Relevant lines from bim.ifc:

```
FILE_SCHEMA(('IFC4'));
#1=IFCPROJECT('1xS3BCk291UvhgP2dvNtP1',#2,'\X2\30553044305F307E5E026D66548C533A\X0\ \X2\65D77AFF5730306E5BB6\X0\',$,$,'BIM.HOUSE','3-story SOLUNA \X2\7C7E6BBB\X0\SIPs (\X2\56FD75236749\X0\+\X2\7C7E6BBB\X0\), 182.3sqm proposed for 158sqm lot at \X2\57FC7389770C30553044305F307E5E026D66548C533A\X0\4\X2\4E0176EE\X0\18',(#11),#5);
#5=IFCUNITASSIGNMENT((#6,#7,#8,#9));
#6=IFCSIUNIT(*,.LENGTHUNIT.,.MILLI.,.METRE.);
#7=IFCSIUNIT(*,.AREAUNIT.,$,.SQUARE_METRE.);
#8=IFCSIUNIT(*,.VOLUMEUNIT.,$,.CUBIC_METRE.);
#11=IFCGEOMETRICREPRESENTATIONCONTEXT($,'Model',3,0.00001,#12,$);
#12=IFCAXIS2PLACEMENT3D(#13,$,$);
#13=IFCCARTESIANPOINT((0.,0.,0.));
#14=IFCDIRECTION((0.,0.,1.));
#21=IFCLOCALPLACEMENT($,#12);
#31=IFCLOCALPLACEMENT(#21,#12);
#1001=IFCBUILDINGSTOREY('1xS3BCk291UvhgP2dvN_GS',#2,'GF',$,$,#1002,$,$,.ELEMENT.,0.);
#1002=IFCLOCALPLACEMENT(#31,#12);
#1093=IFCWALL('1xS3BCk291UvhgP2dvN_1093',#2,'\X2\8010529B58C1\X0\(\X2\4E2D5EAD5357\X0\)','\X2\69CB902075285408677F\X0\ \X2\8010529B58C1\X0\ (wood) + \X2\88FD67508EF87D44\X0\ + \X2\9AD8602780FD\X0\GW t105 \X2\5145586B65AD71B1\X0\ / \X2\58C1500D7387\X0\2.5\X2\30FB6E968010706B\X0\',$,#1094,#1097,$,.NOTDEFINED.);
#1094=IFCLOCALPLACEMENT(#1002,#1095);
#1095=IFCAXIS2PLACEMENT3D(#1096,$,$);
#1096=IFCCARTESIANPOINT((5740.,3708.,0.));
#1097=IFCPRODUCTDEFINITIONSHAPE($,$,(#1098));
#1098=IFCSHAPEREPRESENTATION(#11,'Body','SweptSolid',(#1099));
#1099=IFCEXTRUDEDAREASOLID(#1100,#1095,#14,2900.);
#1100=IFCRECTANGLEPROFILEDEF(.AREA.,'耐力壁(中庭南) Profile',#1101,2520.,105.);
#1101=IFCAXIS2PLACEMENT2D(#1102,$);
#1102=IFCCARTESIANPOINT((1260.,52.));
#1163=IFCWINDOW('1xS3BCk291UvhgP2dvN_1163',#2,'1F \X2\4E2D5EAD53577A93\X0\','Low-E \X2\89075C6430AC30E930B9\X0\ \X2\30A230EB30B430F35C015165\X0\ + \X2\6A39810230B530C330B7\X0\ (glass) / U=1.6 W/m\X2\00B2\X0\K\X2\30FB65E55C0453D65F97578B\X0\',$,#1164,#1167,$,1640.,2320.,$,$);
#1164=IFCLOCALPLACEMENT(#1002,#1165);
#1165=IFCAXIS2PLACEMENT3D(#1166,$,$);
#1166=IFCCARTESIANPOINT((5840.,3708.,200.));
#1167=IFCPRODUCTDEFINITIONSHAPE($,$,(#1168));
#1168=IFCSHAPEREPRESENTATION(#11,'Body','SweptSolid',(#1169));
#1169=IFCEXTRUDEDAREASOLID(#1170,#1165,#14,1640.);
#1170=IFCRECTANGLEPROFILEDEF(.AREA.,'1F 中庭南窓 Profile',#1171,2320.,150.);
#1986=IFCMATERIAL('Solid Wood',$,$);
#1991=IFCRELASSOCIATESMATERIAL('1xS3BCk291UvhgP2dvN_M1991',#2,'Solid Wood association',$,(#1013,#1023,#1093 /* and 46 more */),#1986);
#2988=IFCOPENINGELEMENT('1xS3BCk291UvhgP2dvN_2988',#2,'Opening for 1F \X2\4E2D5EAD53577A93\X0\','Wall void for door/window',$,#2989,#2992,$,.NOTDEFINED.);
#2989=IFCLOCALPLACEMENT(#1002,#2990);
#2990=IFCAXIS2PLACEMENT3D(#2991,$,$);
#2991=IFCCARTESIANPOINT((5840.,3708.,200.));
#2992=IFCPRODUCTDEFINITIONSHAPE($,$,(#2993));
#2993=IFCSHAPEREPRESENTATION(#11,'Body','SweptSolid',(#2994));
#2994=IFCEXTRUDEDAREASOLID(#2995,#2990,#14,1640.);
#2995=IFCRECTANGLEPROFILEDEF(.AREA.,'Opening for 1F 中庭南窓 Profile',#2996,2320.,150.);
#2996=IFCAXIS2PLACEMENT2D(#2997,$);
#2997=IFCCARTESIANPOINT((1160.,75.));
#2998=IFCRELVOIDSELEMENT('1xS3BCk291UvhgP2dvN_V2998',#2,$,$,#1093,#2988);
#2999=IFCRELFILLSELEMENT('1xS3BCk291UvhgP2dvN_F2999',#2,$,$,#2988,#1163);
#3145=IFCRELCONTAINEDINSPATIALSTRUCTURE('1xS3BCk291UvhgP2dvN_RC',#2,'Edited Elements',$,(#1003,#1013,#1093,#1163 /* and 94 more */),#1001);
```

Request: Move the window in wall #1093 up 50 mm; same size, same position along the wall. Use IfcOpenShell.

```python
import numpy as np
import ifcopenshell
import ifcopenshell.api.geometry
import ifcopenshell.util.placement
import ifcopenshell.util.unit

model = ifcopenshell.open("bim.ifc")
unit_scale = ifcopenshell.util.unit.calculate_unit_scale(model)

window = model.by_guid("1xS3BCk291UvhgP2dvN_1163")
opening = window.FillsVoids[0].RelatingOpeningElement
dz = 50.0

shift = np.array([0.0, 0.0, dz])
# The window is not placed relative to its opening, so move both.
for product in (opening, window):
    matrix = ifcopenshell.util.placement.get_local_placement(product.ObjectPlacement)
    matrix[:3, 3] += shift
    ifcopenshell.api.geometry.edit_object_placement(model, product=product, matrix=matrix, is_si=False)

print(f"moved by {dz * unit_scale:+.3f} m")

model.write("bim-out.ifc")
```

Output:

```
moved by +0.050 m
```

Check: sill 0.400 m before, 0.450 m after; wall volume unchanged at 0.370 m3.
